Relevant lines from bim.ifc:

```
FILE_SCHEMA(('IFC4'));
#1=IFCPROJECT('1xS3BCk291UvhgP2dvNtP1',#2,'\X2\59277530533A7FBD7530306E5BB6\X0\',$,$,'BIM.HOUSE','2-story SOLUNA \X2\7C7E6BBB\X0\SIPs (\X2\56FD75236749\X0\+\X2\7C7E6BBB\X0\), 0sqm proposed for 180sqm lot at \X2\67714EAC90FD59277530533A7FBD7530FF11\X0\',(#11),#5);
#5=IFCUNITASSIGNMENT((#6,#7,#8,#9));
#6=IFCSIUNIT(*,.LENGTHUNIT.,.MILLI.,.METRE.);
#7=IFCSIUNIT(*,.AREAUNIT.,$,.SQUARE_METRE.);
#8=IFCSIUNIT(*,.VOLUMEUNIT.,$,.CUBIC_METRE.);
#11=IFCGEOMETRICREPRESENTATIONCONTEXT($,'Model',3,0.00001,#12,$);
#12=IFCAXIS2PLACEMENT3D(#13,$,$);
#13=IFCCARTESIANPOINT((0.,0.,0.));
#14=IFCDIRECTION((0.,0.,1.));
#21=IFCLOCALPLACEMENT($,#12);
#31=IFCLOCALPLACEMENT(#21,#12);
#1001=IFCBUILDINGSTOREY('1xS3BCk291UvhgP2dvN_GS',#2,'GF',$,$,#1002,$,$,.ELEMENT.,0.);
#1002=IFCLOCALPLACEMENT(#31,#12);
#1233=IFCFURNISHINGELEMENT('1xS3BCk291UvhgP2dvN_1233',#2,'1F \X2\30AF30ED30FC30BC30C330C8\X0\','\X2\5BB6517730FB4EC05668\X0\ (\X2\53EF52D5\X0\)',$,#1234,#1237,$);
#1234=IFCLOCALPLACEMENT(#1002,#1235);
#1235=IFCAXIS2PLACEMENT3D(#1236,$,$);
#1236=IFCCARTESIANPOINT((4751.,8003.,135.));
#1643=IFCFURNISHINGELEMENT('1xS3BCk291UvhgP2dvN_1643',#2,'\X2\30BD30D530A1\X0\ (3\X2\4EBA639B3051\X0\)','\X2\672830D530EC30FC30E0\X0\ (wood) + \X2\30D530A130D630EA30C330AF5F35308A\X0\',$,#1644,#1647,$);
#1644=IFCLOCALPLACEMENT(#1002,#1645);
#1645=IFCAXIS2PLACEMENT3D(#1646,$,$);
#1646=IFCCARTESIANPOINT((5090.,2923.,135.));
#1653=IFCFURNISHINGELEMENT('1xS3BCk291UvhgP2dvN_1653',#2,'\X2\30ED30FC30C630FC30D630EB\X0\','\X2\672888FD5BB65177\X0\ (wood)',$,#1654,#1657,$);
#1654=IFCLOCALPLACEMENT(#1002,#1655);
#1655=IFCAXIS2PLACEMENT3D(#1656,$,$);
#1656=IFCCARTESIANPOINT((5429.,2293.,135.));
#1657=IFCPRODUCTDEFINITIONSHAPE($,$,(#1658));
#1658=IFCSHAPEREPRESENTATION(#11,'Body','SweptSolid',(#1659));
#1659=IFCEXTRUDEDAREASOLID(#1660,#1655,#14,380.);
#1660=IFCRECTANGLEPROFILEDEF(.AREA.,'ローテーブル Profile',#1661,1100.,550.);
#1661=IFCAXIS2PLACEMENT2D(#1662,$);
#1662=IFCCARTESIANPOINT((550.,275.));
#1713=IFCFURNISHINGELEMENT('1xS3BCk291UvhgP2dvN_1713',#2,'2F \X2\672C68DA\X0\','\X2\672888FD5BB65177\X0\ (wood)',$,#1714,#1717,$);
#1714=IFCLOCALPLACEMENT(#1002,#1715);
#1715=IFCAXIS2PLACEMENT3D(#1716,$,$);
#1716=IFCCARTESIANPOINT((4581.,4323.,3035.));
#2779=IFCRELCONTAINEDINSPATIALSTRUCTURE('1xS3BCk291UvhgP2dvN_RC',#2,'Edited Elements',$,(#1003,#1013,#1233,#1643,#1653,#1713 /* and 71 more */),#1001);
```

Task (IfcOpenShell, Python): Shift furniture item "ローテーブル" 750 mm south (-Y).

```python
import ifcopenshell
import ifcopenshell.api.geometry
import ifcopenshell.util.placement
import ifcopenshell.util.unit

model = ifcopenshell.open("bim.ifc")
unit_scale = ifcopenshell.util.unit.calculate_unit_scale(model)

item = model.by_id(1653)
matrix = ifcopenshell.util.placement.get_local_placement(item.ObjectPlacement)
matrix[1, 3] -= 0.75 / unit_scale
ifcopenshell.api.geometry.edit_object_placement(model, product=item, matrix=matrix, is_si=False)

print(ifcopenshell.util.placement.get_local_placement(item.ObjectPlacement).round(3) + 0.0)

model.write("bim_edited.ifc")
```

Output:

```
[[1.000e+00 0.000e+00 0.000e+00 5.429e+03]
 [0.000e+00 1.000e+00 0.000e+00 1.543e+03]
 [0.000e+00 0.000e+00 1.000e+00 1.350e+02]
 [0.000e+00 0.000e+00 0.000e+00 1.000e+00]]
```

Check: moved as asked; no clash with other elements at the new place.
